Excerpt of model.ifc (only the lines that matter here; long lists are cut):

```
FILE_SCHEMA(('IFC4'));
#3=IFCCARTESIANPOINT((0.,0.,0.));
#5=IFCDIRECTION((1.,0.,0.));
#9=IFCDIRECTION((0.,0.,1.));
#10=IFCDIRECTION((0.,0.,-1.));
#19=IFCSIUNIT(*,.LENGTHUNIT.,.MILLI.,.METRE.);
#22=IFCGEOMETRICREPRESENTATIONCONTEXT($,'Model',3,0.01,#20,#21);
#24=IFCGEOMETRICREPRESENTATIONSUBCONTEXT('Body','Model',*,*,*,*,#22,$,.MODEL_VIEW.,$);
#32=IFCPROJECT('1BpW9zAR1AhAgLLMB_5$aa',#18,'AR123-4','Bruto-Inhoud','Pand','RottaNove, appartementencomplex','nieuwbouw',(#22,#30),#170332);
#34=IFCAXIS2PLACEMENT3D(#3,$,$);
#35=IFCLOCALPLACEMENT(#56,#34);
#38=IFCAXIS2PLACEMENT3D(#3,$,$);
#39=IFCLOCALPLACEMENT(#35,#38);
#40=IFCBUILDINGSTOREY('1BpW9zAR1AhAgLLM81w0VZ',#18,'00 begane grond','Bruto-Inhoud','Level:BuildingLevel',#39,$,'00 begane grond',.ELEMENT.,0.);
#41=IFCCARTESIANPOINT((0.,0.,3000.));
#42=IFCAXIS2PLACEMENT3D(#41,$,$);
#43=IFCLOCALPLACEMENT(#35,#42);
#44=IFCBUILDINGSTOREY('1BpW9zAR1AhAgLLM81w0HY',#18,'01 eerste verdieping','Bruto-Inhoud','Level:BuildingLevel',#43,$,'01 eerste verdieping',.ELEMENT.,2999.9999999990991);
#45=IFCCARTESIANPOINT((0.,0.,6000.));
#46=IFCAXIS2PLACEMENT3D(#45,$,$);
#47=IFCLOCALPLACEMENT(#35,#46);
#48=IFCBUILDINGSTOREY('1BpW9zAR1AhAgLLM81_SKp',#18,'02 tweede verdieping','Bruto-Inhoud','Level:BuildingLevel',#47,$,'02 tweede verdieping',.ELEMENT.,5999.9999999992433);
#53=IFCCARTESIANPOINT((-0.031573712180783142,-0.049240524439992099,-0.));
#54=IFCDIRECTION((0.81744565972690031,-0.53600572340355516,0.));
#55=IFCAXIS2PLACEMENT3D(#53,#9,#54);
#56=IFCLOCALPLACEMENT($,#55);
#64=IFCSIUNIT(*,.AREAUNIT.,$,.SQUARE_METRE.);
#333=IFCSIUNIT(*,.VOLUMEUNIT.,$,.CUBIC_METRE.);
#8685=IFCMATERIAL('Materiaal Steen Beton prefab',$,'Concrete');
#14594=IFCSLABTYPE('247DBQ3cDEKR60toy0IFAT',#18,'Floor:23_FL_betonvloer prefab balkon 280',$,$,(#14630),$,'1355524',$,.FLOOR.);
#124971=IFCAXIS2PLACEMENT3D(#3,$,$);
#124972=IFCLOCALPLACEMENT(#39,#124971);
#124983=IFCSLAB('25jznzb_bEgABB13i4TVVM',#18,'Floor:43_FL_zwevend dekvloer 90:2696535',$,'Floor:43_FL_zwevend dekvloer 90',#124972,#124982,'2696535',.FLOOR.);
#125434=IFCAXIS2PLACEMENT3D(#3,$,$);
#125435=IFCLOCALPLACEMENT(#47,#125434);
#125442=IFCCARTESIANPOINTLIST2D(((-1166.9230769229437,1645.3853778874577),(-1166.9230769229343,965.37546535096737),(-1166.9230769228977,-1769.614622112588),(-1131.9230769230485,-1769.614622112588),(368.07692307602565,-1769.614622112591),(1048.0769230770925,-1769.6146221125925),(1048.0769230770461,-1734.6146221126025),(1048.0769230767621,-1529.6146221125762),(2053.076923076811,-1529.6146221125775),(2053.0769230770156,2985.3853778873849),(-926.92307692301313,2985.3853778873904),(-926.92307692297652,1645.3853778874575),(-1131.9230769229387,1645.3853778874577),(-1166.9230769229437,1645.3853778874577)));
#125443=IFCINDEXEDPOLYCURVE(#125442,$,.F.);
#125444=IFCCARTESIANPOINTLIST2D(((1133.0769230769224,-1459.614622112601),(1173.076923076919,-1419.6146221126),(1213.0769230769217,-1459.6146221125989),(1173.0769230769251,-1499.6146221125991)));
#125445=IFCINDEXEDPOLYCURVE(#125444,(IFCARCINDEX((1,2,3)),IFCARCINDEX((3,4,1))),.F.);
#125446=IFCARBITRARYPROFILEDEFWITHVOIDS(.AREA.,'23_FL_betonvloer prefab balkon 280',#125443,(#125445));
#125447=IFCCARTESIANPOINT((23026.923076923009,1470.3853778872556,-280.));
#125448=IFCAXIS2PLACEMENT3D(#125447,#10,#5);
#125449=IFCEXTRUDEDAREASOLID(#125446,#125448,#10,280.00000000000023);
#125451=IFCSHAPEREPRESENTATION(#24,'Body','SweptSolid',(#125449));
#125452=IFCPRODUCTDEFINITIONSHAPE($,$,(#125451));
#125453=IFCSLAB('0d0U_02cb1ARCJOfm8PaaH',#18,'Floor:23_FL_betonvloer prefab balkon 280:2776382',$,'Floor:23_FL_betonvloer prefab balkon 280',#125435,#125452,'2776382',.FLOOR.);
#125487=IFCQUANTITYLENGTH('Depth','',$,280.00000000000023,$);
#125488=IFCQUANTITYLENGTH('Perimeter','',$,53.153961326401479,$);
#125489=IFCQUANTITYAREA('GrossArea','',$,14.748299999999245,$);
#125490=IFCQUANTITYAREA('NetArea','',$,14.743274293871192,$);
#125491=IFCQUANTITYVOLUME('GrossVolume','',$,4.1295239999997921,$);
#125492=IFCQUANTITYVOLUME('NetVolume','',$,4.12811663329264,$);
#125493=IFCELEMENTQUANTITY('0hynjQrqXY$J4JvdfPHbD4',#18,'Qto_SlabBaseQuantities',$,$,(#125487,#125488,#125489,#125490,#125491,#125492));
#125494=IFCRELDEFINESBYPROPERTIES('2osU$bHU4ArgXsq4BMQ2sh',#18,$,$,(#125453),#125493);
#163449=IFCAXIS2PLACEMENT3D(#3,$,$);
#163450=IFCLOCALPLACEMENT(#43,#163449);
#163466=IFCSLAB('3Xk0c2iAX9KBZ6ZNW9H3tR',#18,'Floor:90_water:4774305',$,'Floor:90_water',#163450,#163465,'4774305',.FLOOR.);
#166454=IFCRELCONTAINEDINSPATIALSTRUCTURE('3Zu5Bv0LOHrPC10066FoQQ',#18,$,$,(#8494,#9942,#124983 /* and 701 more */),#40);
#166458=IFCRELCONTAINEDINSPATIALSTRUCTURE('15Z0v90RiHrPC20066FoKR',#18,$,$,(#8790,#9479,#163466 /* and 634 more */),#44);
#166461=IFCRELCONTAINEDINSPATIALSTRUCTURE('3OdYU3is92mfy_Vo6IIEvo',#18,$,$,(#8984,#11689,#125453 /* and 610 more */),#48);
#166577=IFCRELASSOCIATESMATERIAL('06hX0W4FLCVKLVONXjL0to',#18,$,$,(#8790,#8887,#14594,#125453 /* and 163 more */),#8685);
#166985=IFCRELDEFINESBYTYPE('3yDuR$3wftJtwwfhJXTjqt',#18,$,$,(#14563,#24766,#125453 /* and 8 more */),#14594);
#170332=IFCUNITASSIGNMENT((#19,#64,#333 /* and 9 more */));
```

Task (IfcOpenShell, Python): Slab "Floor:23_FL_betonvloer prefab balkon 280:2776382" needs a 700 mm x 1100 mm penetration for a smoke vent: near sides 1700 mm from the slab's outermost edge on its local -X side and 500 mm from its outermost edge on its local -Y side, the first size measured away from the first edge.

```python
import numpy as np
import ifcopenshell
import ifcopenshell.api.feature
import ifcopenshell.api.geometry
import ifcopenshell.api.pset
import ifcopenshell.api.root
import ifcopenshell.geom
import ifcopenshell.util.element
import ifcopenshell.util.placement
import ifcopenshell.util.representation
import ifcopenshell.util.shape
import ifcopenshell.util.unit

model = ifcopenshell.open("model.ifc")
unit_scale = ifcopenshell.util.unit.calculate_unit_scale(model)
area_scale = ifcopenshell.util.unit.calculate_unit_scale(model, "AREAUNIT")
volume_scale = ifcopenshell.util.unit.calculate_unit_scale(model, "VOLUMEUNIT")
settings = ifcopenshell.geom.settings()


def volume(element):
    """Net volume in cubic metres, openings subtracted."""
    shape = ifcopenshell.geom.create_shape(settings, element)
    return ifcopenshell.util.shape.get_volume(shape.geometry)


slab = model.by_guid("0d0U_02cb1ARCJOfm8PaaH")
before = volume(slab)

# Extent in the slab's own axes, in metres. The edges named are its -X and -Y sides.
slab_shape = ifcopenshell.geom.create_shape(settings, slab)
vertices = ifcopenshell.util.shape.get_vertices(slab_shape.geometry)
x_min, y_min, bottom = vertices.min(axis=0)
top = vertices[:, 2].max()

opening = ifcopenshell.api.root.create_entity(model, ifc_class="IfcOpeningElement", name="Smoke vent opening", predefined_type="OPENING")
context = ifcopenshell.util.representation.get_context(model, "Model", "Body", "MODEL_VIEW")
width, depth = 0.7, 1.1
outline = [(0.0, 0.0), (width, 0.0), (width, depth), (0.0, depth), (0.0, 0.0)]
# Overshoot both faces by 50 mm so the cut is clean.
shape = ifcopenshell.api.geometry.add_slab_representation(
    model, context=context, depth=top - bottom + 0.1, polyline=outline
)
ifcopenshell.api.geometry.assign_representation(model, product=opening, representation=shape)

matrix = ifcopenshell.util.placement.get_local_placement(slab.ObjectPlacement)
matrix[:, 3] = matrix @ np.append(np.array([x_min + 1.7, y_min + 0.5, bottom - 0.05]) / unit_scale, 1.0)
ifcopenshell.api.geometry.edit_object_placement(model, product=opening, matrix=matrix, is_si=False)
ifcopenshell.api.feature.add_feature(model, feature=opening, element=slab)

after = volume(slab)

# Update the slab's stored quantities.
qto = model.by_id(ifcopenshell.util.element.get_pset(slab, "Qto_SlabBaseQuantities", should_inherit=False)["id"])
ifcopenshell.api.pset.edit_qto(model, qto=qto, properties={
    "NetArea": after / (top - bottom) / area_scale,
    "NetVolume": after / volume_scale,
})

print(f"slab volume {before:.3f} -> {after:.3f} m3")

model.write("model_edited.ifc")
```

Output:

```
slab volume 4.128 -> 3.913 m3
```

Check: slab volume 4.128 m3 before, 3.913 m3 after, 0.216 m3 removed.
